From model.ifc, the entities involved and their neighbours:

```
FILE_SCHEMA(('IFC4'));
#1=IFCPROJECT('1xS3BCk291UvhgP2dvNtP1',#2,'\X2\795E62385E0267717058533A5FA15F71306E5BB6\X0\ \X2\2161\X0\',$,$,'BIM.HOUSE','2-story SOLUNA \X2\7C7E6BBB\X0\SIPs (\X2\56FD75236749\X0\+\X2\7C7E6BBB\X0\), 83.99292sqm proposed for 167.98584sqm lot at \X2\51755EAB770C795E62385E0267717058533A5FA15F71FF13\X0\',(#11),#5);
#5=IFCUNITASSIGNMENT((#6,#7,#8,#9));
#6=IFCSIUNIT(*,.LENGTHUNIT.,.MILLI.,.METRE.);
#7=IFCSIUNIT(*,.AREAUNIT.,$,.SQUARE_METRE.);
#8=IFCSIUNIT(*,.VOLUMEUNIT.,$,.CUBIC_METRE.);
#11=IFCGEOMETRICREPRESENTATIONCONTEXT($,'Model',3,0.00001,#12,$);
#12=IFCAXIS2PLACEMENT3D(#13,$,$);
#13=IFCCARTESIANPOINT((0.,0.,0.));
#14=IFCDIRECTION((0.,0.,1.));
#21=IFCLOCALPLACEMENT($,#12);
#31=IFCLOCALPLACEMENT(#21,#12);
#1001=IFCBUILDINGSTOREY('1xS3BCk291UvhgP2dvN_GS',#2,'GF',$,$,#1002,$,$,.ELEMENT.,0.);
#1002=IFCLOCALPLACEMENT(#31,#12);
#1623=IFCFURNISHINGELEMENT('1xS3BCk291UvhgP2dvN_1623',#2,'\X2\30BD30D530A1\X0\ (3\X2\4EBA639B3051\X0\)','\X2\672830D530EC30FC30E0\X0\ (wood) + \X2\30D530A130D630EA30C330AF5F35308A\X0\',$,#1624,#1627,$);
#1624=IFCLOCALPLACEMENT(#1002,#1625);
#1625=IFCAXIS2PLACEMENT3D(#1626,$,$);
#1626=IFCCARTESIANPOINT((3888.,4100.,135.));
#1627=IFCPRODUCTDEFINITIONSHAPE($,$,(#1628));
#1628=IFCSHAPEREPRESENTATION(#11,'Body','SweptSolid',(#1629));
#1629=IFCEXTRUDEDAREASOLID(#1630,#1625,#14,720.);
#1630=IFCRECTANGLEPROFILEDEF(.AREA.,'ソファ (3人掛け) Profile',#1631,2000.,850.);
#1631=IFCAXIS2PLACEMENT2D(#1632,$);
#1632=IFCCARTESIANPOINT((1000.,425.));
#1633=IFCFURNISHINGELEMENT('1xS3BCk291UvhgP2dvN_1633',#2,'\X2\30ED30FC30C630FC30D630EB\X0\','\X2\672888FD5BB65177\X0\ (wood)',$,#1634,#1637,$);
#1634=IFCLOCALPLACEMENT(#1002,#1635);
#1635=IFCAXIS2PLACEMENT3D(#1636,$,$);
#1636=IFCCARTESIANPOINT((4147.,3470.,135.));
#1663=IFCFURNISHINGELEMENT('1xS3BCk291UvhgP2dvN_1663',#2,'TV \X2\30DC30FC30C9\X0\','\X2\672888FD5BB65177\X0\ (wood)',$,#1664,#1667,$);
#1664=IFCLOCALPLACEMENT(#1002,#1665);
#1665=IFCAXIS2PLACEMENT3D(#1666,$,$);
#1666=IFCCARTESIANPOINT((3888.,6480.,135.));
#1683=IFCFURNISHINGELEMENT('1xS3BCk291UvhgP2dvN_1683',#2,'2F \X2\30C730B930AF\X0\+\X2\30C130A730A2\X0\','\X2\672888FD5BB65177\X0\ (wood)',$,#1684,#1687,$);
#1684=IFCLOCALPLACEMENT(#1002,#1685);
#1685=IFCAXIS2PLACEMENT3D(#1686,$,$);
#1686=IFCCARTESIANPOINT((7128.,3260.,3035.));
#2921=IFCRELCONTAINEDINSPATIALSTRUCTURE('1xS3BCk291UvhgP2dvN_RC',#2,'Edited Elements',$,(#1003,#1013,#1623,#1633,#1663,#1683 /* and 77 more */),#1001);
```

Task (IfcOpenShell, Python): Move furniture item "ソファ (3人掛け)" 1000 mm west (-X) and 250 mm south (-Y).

```python
import ifcopenshell
import ifcopenshell.api.geometry
import ifcopenshell.util.placement

model = ifcopenshell.open("model.ifc")

item = model.by_guid("1xS3BCk291UvhgP2dvN_1623")
matrix = ifcopenshell.util.placement.get_local_placement(item.ObjectPlacement)
matrix[0, 3] -= 1000.0
matrix[1, 3] -= 250.0
ifcopenshell.api.geometry.edit_object_placement(model, product=item, matrix=matrix, is_si=False)

print(ifcopenshell.util.placement.get_local_placement(item.ObjectPlacement).round(3) + 0.0)

model.write("model_rev.ifc")
```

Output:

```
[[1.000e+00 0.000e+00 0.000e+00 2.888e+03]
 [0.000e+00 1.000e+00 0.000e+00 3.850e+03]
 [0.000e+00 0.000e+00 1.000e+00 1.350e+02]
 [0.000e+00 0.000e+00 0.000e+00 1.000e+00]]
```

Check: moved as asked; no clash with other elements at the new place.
